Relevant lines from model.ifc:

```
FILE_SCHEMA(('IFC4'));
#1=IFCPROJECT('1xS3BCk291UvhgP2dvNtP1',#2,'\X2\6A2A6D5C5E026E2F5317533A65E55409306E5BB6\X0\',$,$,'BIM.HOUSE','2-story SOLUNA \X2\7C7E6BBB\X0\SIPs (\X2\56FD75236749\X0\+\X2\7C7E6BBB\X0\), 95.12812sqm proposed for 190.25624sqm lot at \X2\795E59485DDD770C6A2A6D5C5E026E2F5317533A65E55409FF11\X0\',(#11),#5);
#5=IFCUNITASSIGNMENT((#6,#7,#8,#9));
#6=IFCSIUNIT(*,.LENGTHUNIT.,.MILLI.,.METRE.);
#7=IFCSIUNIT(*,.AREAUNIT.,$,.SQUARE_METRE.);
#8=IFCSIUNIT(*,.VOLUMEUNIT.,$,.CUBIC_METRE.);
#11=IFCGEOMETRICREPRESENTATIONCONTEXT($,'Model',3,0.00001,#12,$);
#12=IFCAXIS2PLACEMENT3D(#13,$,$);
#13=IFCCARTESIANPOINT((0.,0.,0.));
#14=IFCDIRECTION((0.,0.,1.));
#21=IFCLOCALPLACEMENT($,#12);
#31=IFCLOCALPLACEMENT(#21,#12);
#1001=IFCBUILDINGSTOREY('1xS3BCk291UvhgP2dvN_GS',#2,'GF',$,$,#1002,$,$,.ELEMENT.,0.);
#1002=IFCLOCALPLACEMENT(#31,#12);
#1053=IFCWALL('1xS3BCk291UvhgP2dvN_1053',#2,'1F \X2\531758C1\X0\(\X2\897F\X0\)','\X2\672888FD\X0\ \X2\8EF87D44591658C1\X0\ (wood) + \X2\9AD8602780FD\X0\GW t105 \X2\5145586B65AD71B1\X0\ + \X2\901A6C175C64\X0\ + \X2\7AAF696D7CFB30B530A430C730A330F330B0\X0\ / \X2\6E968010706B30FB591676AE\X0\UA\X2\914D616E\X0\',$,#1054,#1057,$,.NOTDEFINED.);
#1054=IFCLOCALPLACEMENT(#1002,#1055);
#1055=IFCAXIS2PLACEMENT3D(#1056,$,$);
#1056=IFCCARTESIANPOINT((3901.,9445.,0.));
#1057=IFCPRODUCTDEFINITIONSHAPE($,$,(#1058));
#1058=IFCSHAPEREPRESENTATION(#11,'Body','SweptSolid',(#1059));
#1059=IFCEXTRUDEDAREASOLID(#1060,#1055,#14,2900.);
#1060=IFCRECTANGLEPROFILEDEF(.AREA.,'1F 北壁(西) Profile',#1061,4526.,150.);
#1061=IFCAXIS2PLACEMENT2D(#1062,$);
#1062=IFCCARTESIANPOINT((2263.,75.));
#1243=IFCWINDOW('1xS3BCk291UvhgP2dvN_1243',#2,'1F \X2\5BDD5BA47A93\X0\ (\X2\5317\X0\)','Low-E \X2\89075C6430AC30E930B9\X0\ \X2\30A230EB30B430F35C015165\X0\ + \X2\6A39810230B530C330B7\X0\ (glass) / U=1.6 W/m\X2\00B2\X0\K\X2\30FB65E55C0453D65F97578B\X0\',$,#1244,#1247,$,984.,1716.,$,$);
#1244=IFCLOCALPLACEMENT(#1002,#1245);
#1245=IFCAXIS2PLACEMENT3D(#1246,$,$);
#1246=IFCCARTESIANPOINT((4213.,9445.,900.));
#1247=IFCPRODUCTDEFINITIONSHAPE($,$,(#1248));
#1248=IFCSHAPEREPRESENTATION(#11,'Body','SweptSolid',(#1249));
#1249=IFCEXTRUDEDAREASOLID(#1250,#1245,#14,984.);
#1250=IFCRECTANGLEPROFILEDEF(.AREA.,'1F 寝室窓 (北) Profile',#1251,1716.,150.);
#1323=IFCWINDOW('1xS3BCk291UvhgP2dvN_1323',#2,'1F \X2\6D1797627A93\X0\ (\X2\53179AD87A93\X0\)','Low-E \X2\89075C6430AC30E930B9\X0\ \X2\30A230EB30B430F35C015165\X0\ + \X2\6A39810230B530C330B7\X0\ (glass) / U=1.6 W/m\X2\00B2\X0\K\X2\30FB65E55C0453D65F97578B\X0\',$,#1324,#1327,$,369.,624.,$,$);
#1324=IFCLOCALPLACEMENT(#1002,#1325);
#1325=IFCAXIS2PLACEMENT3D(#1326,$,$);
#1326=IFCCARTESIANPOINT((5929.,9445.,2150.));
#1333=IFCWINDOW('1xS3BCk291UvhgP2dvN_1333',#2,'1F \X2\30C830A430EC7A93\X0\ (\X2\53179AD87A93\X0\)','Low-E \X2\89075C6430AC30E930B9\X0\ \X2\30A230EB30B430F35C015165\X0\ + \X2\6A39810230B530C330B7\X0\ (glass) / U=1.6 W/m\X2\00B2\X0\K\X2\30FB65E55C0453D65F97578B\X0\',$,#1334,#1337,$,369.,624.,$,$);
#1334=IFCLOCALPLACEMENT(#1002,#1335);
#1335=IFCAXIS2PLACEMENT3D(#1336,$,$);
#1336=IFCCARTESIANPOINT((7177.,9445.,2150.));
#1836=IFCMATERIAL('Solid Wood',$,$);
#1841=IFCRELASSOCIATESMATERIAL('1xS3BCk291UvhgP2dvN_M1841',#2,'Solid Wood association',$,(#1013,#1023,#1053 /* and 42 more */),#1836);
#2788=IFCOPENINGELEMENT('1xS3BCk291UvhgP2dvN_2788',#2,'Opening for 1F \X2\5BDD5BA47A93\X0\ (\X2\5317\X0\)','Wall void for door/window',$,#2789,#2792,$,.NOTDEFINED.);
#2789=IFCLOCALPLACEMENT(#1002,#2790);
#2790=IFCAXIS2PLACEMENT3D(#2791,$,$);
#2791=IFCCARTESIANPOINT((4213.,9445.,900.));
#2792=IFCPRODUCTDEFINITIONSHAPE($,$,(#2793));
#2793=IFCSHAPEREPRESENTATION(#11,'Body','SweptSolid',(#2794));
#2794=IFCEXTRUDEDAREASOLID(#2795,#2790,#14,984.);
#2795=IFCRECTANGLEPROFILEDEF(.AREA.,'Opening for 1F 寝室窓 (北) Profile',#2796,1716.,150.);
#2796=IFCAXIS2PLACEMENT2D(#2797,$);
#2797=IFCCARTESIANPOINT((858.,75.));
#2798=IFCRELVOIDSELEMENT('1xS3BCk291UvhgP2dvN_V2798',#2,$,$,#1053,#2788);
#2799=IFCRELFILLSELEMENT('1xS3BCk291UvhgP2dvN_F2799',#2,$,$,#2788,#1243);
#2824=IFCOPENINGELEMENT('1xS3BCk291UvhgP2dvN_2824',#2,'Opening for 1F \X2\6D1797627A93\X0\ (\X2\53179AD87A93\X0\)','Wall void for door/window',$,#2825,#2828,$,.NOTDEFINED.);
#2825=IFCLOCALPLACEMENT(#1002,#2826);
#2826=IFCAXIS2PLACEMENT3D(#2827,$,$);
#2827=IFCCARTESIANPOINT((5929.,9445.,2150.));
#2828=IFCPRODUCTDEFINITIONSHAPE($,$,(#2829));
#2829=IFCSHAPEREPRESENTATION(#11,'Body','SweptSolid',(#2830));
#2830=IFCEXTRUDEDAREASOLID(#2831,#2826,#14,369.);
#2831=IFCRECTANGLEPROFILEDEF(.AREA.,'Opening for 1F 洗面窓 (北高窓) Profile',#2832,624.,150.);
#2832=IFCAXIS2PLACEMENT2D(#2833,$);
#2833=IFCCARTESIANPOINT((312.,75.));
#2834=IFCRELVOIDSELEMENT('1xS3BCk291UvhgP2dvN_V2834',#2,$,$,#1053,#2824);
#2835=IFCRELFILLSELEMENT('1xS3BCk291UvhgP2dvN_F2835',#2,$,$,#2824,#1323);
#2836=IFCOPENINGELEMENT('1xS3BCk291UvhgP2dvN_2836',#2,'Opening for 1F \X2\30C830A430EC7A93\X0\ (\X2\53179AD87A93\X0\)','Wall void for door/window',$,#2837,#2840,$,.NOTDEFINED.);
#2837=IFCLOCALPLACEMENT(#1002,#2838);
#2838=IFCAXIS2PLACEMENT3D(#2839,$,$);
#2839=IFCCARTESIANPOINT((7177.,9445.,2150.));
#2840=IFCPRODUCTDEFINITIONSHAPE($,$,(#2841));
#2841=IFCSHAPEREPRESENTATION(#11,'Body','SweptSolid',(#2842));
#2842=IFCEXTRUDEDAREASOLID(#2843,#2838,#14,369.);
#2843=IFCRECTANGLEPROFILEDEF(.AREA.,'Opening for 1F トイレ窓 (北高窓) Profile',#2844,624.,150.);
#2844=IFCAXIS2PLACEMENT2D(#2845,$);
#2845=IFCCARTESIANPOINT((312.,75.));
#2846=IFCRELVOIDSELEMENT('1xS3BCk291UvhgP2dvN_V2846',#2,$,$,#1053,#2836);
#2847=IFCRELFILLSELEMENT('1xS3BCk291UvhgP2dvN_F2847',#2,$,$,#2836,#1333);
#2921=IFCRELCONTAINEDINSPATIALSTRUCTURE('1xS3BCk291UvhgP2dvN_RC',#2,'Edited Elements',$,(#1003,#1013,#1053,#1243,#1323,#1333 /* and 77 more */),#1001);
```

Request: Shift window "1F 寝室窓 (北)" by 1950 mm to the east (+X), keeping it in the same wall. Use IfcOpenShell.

```python
import ifcopenshell
import ifcopenshell.api.geometry
import ifcopenshell.util.placement
import ifcopenshell.util.unit

model = ifcopenshell.open("model.ifc")
unit_scale = ifcopenshell.util.unit.calculate_unit_scale(model)

window = model.by_guid("1xS3BCk291UvhgP2dvN_1243")
opening = window.FillsVoids[0].RelatingOpeningElement
wall = opening.VoidsElements[0].RelatingBuildingElement

wall_matrix = ifcopenshell.util.placement.get_local_placement(wall.ObjectPlacement)
shift = wall_matrix[:3, 0] * 1.95 / unit_scale
before = ifcopenshell.util.placement.get_local_placement(window.ObjectPlacement)[:3, 3].copy()

# The window is not placed relative to its opening, so move both.
for product in (opening, window):
    matrix = ifcopenshell.util.placement.get_local_placement(product.ObjectPlacement)
    matrix[:3, 3] += shift
    ifcopenshell.api.geometry.edit_object_placement(model, product=product, matrix=matrix, is_si=False)

after = ifcopenshell.util.placement.get_local_placement(window.ObjectPlacement)[:3, 3]
print("window moved by", (after - before).round(3) + 0.0)

model.write("model-out.ifc")
```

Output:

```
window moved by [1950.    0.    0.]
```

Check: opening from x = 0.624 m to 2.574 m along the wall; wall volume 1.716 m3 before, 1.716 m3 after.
